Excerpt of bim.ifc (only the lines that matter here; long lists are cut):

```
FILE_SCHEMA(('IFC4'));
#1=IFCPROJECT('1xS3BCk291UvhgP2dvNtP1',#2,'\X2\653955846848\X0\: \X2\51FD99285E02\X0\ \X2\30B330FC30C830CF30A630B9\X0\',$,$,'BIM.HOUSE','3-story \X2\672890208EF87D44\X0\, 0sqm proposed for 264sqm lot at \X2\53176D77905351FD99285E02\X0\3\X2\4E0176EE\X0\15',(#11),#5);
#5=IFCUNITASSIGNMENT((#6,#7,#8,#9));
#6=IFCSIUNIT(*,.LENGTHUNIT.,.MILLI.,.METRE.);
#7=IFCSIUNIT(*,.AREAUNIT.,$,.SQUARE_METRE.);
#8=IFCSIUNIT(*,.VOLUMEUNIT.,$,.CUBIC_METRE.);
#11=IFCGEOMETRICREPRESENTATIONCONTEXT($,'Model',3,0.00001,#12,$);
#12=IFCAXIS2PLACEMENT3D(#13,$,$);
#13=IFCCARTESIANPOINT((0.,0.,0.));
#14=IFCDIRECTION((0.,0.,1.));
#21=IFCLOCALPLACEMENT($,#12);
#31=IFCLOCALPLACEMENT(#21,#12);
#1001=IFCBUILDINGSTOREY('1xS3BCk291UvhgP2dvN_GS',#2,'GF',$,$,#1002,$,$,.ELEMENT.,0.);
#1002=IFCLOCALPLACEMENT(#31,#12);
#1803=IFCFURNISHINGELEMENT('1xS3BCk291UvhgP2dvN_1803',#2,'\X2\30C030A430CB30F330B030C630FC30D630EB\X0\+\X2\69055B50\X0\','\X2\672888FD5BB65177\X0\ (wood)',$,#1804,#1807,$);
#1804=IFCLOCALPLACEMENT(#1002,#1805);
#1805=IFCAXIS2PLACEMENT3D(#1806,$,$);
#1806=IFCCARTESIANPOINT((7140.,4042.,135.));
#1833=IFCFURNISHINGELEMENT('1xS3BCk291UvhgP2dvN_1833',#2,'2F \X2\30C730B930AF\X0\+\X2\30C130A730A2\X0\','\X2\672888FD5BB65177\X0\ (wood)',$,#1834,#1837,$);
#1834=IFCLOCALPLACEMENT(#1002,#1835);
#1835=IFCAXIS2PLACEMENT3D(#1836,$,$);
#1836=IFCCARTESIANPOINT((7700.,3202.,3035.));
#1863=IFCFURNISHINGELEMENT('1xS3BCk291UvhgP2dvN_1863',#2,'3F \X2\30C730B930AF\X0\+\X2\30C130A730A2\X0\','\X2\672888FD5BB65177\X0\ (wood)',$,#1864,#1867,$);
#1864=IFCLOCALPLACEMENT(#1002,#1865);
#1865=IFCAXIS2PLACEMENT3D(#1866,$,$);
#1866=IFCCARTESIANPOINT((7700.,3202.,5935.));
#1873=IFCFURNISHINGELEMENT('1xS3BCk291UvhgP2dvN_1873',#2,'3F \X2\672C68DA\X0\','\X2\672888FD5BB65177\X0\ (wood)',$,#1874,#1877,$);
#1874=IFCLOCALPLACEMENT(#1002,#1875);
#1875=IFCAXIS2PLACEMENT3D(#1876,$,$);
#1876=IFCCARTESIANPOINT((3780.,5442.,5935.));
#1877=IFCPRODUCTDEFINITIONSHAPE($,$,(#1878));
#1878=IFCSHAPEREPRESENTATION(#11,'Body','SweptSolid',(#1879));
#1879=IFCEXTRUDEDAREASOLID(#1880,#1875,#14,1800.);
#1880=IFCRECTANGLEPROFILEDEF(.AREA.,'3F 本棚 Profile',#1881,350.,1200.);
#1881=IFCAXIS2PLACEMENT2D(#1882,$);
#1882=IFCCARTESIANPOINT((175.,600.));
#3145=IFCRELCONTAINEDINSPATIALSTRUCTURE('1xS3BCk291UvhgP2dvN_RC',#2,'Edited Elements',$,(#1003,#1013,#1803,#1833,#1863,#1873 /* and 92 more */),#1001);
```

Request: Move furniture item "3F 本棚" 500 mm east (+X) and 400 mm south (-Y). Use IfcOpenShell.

```python
import ifcopenshell
import ifcopenshell.api.geometry
import ifcopenshell.util.placement

model = ifcopenshell.open("bim.ifc")

item = model.by_guid("1xS3BCk291UvhgP2dvN_1873")
matrix = ifcopenshell.util.placement.get_local_placement(item.ObjectPlacement)
matrix[0, 3] += 500.0
matrix[1, 3] -= 400.0
ifcopenshell.api.geometry.edit_object_placement(model, product=item, matrix=matrix, is_si=False)

print(ifcopenshell.util.placement.get_local_placement(item.ObjectPlacement).round(3) + 0.0)

model.write("bim-out.ifc")
```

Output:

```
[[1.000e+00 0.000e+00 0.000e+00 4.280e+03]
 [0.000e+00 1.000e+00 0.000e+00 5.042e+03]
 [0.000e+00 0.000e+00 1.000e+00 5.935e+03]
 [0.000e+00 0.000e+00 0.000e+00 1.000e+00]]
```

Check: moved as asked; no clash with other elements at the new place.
